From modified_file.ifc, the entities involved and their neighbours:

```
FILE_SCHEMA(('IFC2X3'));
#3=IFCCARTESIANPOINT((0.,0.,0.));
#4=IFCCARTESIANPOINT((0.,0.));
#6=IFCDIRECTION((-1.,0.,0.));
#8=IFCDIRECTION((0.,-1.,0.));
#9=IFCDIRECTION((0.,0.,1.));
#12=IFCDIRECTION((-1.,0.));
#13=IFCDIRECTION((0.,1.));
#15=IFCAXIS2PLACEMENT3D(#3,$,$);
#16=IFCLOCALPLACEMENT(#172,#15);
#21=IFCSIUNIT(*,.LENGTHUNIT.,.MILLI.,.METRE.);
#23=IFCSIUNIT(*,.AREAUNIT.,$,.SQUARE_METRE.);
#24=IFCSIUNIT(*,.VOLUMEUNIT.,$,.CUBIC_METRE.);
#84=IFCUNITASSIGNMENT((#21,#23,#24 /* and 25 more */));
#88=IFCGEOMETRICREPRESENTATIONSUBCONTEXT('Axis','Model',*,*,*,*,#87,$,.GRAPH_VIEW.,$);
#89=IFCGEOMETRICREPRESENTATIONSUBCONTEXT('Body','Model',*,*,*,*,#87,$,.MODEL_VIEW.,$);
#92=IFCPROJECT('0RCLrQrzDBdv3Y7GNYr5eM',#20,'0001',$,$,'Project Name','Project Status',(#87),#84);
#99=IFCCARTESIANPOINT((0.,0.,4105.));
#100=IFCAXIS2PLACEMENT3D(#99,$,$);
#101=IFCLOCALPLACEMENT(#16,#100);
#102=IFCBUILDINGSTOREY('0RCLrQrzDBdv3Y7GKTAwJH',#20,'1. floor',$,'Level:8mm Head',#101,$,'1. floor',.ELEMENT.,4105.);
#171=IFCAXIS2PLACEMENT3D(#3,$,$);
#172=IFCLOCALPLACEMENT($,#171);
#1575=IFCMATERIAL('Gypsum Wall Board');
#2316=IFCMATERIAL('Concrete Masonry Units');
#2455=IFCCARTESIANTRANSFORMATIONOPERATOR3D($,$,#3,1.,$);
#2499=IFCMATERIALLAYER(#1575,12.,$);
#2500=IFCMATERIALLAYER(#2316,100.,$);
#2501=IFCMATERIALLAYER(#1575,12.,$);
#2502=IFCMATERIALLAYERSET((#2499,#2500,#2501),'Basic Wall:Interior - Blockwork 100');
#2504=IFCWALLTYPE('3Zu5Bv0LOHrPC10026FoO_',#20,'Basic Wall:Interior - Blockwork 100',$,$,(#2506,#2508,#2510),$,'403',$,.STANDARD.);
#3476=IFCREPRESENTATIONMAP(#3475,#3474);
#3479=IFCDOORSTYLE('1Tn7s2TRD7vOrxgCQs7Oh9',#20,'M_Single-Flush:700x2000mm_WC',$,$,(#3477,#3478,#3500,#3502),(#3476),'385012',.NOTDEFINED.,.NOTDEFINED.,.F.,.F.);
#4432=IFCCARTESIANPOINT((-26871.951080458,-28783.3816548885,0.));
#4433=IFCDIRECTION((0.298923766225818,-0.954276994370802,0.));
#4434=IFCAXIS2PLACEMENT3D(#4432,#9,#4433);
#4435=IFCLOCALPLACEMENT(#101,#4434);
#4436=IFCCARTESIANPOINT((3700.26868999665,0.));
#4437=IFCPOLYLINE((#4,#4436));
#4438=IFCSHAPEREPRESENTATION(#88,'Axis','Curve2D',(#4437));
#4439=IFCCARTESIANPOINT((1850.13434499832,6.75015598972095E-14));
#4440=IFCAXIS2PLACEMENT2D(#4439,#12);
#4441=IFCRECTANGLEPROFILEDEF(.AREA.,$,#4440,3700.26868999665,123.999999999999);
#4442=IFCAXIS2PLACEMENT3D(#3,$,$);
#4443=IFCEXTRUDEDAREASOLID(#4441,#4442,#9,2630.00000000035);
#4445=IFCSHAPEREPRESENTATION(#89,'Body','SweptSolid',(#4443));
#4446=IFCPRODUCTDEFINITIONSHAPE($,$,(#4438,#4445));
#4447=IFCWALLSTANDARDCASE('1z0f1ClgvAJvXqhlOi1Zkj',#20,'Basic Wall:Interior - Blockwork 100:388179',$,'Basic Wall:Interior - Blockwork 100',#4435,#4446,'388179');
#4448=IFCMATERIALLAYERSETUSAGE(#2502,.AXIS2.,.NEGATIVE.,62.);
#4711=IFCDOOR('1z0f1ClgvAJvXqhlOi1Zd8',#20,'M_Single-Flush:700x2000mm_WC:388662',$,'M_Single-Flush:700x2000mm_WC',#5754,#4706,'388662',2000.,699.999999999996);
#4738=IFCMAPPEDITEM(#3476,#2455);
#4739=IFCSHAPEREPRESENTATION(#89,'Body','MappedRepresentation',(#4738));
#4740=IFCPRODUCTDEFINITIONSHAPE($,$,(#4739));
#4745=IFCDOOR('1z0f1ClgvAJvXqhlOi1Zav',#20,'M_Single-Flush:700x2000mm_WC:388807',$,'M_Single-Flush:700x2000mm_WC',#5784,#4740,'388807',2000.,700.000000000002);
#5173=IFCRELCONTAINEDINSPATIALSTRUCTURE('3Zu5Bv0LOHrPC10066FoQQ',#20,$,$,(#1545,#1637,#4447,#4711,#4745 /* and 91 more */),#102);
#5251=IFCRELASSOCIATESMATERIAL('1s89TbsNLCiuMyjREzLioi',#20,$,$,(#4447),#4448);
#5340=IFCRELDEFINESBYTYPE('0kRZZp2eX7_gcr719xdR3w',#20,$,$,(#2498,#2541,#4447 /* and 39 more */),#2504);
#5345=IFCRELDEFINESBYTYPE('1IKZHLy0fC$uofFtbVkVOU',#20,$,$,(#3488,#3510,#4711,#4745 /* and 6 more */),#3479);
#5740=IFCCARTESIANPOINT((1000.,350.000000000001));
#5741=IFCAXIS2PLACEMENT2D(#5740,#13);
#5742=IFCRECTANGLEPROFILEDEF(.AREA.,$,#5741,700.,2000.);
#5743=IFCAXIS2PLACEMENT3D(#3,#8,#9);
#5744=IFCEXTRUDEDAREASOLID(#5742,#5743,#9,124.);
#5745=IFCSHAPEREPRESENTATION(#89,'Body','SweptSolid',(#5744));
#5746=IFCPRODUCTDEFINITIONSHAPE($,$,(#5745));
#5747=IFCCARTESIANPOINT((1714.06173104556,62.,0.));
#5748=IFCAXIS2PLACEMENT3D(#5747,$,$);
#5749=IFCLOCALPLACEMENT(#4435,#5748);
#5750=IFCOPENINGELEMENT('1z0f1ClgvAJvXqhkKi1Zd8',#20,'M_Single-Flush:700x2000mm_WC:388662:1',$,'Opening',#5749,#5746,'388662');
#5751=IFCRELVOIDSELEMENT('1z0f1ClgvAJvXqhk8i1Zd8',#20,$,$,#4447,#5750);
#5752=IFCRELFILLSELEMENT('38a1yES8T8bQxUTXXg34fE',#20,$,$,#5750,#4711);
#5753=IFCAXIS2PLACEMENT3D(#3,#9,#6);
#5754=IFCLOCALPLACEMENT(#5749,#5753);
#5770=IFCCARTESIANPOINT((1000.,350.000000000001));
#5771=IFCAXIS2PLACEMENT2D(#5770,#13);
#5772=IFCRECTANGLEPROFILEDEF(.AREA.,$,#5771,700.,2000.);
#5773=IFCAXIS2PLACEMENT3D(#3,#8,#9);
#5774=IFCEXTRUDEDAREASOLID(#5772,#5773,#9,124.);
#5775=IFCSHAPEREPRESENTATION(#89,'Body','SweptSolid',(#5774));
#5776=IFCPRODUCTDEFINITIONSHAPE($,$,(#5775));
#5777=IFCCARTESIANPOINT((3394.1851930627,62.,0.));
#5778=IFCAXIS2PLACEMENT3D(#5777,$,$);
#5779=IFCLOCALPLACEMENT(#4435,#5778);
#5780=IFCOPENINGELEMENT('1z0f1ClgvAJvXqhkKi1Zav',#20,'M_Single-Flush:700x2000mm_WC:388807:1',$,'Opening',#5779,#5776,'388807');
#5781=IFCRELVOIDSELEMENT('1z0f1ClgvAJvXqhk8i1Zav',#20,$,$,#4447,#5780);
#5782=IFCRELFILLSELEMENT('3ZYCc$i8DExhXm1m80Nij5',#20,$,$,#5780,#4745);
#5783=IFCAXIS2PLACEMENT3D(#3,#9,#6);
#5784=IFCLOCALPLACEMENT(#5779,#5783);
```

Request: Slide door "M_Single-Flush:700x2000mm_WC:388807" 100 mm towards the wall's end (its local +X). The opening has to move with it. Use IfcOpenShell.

```python
import ifcopenshell
import ifcopenshell.api.geometry
import ifcopenshell.util.placement
import ifcopenshell.util.unit

model = ifcopenshell.open("modified_file.ifc")
unit_scale = ifcopenshell.util.unit.calculate_unit_scale(model)

door = model.by_guid("1z0f1ClgvAJvXqhlOi1Zav")
opening = door.FillsVoids[0].RelatingOpeningElement
wall = opening.VoidsElements[0].RelatingBuildingElement

wall_matrix = ifcopenshell.util.placement.get_local_placement(wall.ObjectPlacement)
shift = wall_matrix[:3, 0] * 0.1 / unit_scale
before = ifcopenshell.util.placement.get_local_placement(door.ObjectPlacement)[:3, 3].copy()

# The door is placed relative to its opening, so it follows when the opening moves.
matrix = ifcopenshell.util.placement.get_local_placement(opening.ObjectPlacement)
matrix[:3, 3] += shift
ifcopenshell.api.geometry.edit_object_placement(
    model, product=opening, matrix=matrix, is_si=False, should_transform_children=True
)

after = ifcopenshell.util.placement.get_local_placement(door.ObjectPlacement)[:3, 3]
print("door moved by", (after - before).round(3) + 0.0)

model.write("modified_file_v2.ifc")
```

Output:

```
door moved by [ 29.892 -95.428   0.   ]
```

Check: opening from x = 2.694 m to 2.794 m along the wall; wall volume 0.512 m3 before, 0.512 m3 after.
